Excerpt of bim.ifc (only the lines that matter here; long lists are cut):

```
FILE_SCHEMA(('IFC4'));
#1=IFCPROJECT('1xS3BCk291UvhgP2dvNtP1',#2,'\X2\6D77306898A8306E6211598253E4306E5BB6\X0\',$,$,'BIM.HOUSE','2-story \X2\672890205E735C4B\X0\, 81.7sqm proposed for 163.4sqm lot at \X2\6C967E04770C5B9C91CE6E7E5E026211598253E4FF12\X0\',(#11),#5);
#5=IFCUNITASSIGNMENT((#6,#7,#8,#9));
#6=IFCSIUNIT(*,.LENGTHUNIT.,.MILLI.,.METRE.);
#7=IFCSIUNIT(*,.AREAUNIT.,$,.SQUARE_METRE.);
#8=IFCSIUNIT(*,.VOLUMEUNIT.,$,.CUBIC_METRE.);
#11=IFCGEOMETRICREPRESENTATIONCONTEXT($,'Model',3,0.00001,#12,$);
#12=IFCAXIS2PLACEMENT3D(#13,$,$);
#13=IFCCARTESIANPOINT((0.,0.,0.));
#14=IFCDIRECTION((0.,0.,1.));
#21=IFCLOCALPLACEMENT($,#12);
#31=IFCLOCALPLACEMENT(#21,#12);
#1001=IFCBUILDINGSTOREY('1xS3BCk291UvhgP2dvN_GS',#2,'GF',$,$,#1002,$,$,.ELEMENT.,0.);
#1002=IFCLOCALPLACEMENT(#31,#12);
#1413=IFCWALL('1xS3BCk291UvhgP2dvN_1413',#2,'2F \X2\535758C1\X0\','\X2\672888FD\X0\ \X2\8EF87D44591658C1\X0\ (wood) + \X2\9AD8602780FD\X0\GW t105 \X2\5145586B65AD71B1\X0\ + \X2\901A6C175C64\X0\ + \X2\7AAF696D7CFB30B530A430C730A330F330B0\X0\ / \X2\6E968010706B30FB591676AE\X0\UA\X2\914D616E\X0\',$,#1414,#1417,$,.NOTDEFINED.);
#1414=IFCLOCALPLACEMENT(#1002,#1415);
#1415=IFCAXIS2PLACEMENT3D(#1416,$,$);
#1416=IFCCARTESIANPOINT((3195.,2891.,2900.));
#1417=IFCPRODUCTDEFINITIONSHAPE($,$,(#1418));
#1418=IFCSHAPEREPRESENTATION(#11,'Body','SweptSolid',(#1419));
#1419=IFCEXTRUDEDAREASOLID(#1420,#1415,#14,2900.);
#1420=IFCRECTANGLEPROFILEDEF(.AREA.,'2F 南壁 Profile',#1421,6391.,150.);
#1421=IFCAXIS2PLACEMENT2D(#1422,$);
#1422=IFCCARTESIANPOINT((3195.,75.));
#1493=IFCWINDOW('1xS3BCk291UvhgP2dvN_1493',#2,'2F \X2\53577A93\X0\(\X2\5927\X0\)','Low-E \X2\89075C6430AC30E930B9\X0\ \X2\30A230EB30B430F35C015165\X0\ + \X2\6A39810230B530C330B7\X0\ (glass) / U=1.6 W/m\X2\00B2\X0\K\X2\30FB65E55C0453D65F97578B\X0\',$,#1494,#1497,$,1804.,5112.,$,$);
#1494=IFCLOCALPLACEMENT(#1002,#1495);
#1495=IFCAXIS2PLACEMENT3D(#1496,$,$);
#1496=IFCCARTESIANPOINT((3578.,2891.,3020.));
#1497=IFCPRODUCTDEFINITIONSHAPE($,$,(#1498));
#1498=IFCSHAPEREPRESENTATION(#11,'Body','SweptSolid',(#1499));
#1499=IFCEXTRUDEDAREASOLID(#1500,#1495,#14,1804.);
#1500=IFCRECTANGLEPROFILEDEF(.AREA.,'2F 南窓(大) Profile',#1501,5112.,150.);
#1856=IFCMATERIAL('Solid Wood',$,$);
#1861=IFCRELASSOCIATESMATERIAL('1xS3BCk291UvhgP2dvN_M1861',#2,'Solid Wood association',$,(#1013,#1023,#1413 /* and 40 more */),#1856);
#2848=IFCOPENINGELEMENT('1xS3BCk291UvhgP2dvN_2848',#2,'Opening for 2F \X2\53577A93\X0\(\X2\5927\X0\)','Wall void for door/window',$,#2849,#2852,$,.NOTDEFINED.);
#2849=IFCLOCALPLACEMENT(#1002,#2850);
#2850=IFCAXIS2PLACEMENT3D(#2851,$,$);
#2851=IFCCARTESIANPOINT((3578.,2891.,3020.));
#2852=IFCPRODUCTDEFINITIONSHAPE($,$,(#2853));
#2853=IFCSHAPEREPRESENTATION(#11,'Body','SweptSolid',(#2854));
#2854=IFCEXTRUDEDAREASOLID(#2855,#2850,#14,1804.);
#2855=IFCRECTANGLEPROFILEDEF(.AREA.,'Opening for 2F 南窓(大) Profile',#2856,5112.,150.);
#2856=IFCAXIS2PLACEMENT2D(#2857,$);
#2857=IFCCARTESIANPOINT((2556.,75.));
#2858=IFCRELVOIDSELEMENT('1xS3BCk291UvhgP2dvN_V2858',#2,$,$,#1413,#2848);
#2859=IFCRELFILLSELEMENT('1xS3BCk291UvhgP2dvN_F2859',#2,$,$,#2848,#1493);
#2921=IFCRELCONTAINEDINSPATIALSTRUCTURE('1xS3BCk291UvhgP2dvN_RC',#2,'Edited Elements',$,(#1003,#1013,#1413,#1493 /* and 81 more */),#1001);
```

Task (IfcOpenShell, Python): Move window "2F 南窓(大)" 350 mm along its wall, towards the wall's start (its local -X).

```python
import ifcopenshell
import ifcopenshell.api.geometry
import ifcopenshell.util.placement
import ifcopenshell.util.unit

model = ifcopenshell.open("bim.ifc")
unit_scale = ifcopenshell.util.unit.calculate_unit_scale(model)

window = model.by_guid("1xS3BCk291UvhgP2dvN_1493")
opening = window.FillsVoids[0].RelatingOpeningElement
wall = opening.VoidsElements[0].RelatingBuildingElement

wall_matrix = ifcopenshell.util.placement.get_local_placement(wall.ObjectPlacement)
shift = wall_matrix[:3, 0] * -0.35 / unit_scale
before = ifcopenshell.util.placement.get_local_placement(window.ObjectPlacement)[:3, 3].copy()

# The window is not placed relative to its opening, so move both.
for product in (opening, window):
    matrix = ifcopenshell.util.placement.get_local_placement(product.ObjectPlacement)
    matrix[:3, 3] += shift
    ifcopenshell.api.geometry.edit_object_placement(model, product=product, matrix=matrix, is_si=False)

after = ifcopenshell.util.placement.get_local_placement(window.ObjectPlacement)[:3, 3]
print("window moved by", (after - before).round(3) + 0.0)

model.write("bim-out.ifc")
```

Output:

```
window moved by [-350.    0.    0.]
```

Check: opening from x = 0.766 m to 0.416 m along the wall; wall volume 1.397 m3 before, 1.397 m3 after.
